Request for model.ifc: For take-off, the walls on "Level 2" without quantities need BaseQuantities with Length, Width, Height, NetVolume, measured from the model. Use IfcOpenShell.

First a look at what the model holds.

```python
import ifcopenshell
import ifcopenshell.util.element
import ifcopenshell.util.unit

model = ifcopenshell.open("model.ifc")
print(model.schema)
for unit_type in ("LENGTHUNIT", "AREAUNIT", "VOLUMEUNIT"):
    print(unit_type, ifcopenshell.util.unit.calculate_unit_scale(model, unit_type))
storey = next(s for s in model.by_type("IfcBuildingStorey") if s.Name == "Level 2")
walls = [e for e in ifcopenshell.util.element.get_decomposition(storey) if e.is_a("IfcWall")]
for e in sorted(walls, key=lambda e: e.id()):
    print(e.id(), e.is_a(), e.Name, list(ifcopenshell.util.element.get_psets(e, qtos_only=True)), sep=" | ")
```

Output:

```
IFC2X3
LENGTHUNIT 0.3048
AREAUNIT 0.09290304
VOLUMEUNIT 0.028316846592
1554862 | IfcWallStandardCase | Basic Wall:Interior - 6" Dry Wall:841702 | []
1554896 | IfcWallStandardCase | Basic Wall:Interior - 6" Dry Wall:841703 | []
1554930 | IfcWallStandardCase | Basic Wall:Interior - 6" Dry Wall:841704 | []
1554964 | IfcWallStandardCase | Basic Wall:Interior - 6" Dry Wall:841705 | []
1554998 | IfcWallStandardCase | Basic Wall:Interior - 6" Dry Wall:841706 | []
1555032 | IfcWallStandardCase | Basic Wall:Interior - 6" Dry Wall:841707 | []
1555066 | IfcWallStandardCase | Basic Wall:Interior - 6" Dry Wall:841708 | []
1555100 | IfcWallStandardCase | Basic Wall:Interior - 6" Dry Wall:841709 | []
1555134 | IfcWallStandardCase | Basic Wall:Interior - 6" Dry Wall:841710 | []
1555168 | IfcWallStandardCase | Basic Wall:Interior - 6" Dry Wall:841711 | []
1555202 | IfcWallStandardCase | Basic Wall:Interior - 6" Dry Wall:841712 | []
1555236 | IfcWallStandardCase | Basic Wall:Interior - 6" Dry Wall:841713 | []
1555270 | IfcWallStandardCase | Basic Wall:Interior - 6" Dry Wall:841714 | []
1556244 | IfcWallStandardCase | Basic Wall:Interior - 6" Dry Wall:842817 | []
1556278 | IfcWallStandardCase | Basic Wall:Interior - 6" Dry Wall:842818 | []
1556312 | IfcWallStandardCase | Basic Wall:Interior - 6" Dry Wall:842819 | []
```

```python
import ifcopenshell
import ifcopenshell.api.pset
import ifcopenshell.geom
import ifcopenshell.util.element
import ifcopenshell.util.shape
import ifcopenshell.util.unit

model = ifcopenshell.open("model.ifc")
unit_scale = ifcopenshell.util.unit.calculate_unit_scale(model)
volume_scale = ifcopenshell.util.unit.calculate_unit_scale(model, "VOLUMEUNIT")
settings = ifcopenshell.geom.settings()

storey = next(s for s in model.by_type("IfcBuildingStorey") if s.Name == "Level 2")
walls = [e for e in ifcopenshell.util.element.get_decomposition(storey) if e.is_a("IfcWall")]

for e in sorted(walls, key=lambda e: e.id()):
    if ifcopenshell.util.element.get_psets(e, qtos_only=True, should_inherit=False):
        continue
    # Geometry comes back in metres, in the element's own axes.
    shape = ifcopenshell.geom.create_shape(settings, e)
    values = {
        "Length": ifcopenshell.util.shape.get_x(shape.geometry) / unit_scale,
        "Width": ifcopenshell.util.shape.get_y(shape.geometry) / unit_scale,
        "Height": ifcopenshell.util.shape.get_z(shape.geometry) / unit_scale,
        "NetVolume": ifcopenshell.util.shape.get_volume(shape.geometry) / volume_scale,
    }
    qto = ifcopenshell.api.pset.add_qto(model, product=e, name="BaseQuantities")
    ifcopenshell.api.pset.edit_qto(model, qto=qto, properties=values)
    print(e.id(), {k: round(v, 3) for k, v in values.items()})

model.write("model-out.ifc")
```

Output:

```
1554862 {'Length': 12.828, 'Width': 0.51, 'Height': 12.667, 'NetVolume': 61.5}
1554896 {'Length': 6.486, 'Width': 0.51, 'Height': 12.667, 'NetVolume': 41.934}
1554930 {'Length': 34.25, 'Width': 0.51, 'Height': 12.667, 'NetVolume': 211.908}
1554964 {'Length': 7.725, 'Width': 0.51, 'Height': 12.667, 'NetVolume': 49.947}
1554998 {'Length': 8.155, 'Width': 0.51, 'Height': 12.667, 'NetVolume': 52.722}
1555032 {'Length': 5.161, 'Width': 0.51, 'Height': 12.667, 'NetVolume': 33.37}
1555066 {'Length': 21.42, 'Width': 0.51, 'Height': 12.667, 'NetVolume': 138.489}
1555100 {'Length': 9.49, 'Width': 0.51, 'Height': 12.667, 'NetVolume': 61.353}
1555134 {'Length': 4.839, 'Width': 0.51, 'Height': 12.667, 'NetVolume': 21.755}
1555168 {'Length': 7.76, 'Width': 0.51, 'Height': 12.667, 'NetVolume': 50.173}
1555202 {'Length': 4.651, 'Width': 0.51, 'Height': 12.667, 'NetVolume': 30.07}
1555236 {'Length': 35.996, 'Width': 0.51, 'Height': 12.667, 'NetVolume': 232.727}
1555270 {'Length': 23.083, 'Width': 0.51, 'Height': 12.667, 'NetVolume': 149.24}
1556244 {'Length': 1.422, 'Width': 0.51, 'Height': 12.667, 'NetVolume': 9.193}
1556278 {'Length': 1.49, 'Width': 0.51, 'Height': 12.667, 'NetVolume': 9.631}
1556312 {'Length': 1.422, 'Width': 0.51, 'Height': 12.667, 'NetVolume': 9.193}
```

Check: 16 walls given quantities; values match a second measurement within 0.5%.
